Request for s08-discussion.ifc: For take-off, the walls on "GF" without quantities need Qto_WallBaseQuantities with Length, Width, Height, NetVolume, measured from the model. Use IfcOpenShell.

First a look at what the model holds.

```python
import ifcopenshell
import ifcopenshell.util.element
import ifcopenshell.util.unit

model = ifcopenshell.open("s08-discussion.ifc")
print(model.schema)
for unit_type in ("LENGTHUNIT", "AREAUNIT", "VOLUMEUNIT"):
    print(unit_type, ifcopenshell.util.unit.calculate_unit_scale(model, unit_type))
storey = next(s for s in model.by_type("IfcBuildingStorey") if s.Name == "GF")
walls = [e for e in ifcopenshell.util.element.get_decomposition(storey) if e.is_a("IfcWall")]
for e in sorted(walls, key=lambda e: e.id()):
    print(e.id(), e.is_a(), e.Name, list(ifcopenshell.util.element.get_psets(e, qtos_only=True)), sep=" | ")
```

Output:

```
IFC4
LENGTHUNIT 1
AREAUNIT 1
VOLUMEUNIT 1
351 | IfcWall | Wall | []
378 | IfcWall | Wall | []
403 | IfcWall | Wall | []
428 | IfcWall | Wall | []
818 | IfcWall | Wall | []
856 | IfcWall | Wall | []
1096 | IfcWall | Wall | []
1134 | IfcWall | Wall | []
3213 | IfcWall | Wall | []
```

```python
import ifcopenshell
import ifcopenshell.api.pset
import ifcopenshell.geom
import ifcopenshell.util.element
import ifcopenshell.util.shape
import ifcopenshell.util.unit

model = ifcopenshell.open("s08-discussion.ifc")
unit_scale = ifcopenshell.util.unit.calculate_unit_scale(model)
volume_scale = ifcopenshell.util.unit.calculate_unit_scale(model, "VOLUMEUNIT")
settings = ifcopenshell.geom.settings()

storey = next(s for s in model.by_type("IfcBuildingStorey") if s.Name == "GF")
walls = [e for e in ifcopenshell.util.element.get_decomposition(storey) if e.is_a("IfcWall")]

for e in sorted(walls, key=lambda e: e.id()):
    if ifcopenshell.util.element.get_psets(e, qtos_only=True, should_inherit=False):
        continue
    # Geometry comes back in metres, in the element's own axes.
    shape = ifcopenshell.geom.create_shape(settings, e)
    values = {
        "Length": ifcopenshell.util.shape.get_x(shape.geometry) / unit_scale,
        "Width": ifcopenshell.util.shape.get_y(shape.geometry) / unit_scale,
        "Height": ifcopenshell.util.shape.get_z(shape.geometry) / unit_scale,
        "NetVolume": ifcopenshell.util.shape.get_volume(shape.geometry) / volume_scale,
    }
    qto = ifcopenshell.api.pset.add_qto(model, product=e, name="Qto_WallBaseQuantities")
    ifcopenshell.api.pset.edit_qto(model, qto=qto, properties=values)
    print(e.id(), {k: round(v, 3) for k, v in values.items()})

model.write("s08-discussion-out.ifc")
```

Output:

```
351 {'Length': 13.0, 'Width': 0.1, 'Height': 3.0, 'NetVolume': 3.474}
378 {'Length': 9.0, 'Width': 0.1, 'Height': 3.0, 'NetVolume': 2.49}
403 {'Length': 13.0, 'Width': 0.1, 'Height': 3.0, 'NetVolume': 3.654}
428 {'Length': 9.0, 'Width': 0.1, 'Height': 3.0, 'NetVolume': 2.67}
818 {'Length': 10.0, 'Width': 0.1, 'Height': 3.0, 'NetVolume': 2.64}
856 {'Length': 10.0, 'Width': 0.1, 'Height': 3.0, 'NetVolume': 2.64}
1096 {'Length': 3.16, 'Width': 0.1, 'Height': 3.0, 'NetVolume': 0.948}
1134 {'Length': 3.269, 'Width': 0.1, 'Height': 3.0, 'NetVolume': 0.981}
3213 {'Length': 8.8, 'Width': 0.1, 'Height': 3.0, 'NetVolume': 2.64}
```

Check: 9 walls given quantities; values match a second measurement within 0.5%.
